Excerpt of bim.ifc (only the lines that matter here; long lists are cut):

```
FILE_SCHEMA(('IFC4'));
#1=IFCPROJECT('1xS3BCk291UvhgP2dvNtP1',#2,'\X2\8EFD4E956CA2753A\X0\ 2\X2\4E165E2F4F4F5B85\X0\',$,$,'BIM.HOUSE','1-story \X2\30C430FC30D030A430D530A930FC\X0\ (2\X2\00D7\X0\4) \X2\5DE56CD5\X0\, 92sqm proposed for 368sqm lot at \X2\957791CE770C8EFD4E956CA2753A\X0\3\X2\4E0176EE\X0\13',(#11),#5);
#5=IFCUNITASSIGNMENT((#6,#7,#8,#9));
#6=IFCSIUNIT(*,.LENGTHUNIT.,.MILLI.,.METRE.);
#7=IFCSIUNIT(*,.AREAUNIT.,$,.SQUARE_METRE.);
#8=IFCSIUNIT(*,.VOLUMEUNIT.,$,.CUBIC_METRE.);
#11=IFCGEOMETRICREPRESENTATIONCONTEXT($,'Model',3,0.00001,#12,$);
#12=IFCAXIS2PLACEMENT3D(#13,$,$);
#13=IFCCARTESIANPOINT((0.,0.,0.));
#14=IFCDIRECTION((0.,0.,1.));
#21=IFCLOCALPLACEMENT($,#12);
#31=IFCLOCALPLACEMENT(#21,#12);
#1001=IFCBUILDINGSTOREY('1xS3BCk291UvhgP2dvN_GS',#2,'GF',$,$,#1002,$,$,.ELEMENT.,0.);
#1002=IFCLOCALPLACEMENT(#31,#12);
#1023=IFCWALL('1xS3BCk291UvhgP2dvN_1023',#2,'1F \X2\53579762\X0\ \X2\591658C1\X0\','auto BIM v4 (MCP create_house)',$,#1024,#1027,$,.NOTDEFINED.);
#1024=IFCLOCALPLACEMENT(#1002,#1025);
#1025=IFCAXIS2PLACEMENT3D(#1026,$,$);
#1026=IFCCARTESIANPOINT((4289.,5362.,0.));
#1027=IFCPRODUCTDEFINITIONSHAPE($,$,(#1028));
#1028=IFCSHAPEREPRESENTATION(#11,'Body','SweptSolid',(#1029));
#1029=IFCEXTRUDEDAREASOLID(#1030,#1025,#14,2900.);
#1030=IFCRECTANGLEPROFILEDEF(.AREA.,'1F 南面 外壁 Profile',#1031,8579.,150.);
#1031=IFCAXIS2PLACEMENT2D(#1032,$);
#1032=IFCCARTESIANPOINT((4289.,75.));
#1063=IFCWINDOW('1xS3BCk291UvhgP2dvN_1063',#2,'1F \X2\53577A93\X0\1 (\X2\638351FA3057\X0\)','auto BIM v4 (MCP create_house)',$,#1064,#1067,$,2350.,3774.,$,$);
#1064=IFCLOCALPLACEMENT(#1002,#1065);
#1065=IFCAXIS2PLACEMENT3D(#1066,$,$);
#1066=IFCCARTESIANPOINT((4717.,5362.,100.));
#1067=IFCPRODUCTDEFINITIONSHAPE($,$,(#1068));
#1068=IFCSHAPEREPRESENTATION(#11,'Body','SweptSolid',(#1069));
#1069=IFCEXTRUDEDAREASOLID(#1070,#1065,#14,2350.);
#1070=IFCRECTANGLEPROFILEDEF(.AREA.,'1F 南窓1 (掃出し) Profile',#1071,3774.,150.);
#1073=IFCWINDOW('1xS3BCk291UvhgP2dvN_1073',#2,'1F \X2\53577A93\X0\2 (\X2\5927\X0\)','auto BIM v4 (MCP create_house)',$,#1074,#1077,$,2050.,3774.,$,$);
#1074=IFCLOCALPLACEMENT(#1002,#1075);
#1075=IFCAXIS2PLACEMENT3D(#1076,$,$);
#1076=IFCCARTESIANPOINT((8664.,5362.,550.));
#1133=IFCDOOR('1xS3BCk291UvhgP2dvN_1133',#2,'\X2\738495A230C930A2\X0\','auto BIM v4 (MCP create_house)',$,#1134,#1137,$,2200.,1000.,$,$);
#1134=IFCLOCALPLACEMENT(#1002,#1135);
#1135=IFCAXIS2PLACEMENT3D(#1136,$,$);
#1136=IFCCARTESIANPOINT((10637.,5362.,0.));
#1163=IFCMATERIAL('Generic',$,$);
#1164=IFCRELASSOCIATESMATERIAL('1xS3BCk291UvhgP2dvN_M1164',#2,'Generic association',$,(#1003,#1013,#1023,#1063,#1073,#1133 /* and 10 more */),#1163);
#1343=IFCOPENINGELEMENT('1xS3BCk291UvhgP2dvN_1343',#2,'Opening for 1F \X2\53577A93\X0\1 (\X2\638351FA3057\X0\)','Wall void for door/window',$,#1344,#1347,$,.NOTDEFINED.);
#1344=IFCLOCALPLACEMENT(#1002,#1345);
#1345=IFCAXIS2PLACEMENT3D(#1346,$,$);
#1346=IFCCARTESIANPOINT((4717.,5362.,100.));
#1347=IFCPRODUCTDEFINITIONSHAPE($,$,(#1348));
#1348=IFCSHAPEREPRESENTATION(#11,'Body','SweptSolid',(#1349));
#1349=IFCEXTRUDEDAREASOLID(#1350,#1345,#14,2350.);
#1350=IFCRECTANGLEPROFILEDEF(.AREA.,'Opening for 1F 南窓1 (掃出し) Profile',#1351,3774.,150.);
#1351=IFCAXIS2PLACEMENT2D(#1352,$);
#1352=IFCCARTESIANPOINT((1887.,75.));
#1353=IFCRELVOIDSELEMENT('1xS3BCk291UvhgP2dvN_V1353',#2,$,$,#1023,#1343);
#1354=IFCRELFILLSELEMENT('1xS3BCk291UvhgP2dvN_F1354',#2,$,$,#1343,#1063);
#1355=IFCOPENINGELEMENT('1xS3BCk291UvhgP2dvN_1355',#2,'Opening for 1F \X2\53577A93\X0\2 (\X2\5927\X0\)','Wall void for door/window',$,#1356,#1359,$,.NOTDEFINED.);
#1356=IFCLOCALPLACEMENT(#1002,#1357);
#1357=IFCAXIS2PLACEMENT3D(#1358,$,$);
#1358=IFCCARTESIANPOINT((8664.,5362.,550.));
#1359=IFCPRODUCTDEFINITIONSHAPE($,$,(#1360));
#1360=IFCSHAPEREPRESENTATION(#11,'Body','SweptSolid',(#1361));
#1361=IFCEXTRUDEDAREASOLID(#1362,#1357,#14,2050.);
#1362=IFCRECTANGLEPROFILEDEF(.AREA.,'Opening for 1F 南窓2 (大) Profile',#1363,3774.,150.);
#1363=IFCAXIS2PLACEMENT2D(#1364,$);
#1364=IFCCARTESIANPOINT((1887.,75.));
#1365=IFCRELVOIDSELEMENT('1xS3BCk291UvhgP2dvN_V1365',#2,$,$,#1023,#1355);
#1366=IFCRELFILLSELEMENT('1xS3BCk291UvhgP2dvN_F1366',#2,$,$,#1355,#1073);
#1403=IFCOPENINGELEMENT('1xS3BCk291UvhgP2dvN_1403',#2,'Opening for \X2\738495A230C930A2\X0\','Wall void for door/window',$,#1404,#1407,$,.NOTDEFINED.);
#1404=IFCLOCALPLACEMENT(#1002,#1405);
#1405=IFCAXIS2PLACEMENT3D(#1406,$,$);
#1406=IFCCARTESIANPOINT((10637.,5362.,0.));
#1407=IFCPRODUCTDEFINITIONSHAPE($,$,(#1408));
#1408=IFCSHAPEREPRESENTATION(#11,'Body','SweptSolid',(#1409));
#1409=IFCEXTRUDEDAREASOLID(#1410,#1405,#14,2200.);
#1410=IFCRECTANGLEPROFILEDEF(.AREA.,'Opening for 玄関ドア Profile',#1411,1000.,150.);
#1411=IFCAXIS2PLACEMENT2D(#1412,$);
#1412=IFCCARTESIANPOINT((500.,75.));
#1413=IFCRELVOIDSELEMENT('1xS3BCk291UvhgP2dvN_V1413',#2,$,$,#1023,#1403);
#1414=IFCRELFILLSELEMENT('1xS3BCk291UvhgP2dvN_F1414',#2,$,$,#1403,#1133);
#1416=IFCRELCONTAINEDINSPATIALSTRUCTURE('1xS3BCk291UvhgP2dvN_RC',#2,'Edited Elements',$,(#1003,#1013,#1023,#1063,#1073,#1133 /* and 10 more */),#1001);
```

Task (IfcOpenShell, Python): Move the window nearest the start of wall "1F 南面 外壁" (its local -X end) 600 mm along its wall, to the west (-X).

```python
import ifcopenshell
import ifcopenshell.api.geometry
import ifcopenshell.util.placement

model = ifcopenshell.open("bim.ifc")

window = model.by_guid("1xS3BCk291UvhgP2dvN_1063")
opening = window.FillsVoids[0].RelatingOpeningElement
wall = opening.VoidsElements[0].RelatingBuildingElement

wall_matrix = ifcopenshell.util.placement.get_local_placement(wall.ObjectPlacement)
shift = wall_matrix[:3, 0] * -600.0
before = ifcopenshell.util.placement.get_local_placement(window.ObjectPlacement)[:3, 3].copy()

# The window is not placed relative to its opening, so move both.
for product in (opening, window):
    matrix = ifcopenshell.util.placement.get_local_placement(product.ObjectPlacement)
    matrix[:3, 3] += shift
    ifcopenshell.api.geometry.edit_object_placement(model, product=product, matrix=matrix, is_si=False)

after = ifcopenshell.util.placement.get_local_placement(window.ObjectPlacement)[:3, 3]
print("window moved by", (after - before).round(3) + 0.0)

model.write("bim_edited.ifc")
```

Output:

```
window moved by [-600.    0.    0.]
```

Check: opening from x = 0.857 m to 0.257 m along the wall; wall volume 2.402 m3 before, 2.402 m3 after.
